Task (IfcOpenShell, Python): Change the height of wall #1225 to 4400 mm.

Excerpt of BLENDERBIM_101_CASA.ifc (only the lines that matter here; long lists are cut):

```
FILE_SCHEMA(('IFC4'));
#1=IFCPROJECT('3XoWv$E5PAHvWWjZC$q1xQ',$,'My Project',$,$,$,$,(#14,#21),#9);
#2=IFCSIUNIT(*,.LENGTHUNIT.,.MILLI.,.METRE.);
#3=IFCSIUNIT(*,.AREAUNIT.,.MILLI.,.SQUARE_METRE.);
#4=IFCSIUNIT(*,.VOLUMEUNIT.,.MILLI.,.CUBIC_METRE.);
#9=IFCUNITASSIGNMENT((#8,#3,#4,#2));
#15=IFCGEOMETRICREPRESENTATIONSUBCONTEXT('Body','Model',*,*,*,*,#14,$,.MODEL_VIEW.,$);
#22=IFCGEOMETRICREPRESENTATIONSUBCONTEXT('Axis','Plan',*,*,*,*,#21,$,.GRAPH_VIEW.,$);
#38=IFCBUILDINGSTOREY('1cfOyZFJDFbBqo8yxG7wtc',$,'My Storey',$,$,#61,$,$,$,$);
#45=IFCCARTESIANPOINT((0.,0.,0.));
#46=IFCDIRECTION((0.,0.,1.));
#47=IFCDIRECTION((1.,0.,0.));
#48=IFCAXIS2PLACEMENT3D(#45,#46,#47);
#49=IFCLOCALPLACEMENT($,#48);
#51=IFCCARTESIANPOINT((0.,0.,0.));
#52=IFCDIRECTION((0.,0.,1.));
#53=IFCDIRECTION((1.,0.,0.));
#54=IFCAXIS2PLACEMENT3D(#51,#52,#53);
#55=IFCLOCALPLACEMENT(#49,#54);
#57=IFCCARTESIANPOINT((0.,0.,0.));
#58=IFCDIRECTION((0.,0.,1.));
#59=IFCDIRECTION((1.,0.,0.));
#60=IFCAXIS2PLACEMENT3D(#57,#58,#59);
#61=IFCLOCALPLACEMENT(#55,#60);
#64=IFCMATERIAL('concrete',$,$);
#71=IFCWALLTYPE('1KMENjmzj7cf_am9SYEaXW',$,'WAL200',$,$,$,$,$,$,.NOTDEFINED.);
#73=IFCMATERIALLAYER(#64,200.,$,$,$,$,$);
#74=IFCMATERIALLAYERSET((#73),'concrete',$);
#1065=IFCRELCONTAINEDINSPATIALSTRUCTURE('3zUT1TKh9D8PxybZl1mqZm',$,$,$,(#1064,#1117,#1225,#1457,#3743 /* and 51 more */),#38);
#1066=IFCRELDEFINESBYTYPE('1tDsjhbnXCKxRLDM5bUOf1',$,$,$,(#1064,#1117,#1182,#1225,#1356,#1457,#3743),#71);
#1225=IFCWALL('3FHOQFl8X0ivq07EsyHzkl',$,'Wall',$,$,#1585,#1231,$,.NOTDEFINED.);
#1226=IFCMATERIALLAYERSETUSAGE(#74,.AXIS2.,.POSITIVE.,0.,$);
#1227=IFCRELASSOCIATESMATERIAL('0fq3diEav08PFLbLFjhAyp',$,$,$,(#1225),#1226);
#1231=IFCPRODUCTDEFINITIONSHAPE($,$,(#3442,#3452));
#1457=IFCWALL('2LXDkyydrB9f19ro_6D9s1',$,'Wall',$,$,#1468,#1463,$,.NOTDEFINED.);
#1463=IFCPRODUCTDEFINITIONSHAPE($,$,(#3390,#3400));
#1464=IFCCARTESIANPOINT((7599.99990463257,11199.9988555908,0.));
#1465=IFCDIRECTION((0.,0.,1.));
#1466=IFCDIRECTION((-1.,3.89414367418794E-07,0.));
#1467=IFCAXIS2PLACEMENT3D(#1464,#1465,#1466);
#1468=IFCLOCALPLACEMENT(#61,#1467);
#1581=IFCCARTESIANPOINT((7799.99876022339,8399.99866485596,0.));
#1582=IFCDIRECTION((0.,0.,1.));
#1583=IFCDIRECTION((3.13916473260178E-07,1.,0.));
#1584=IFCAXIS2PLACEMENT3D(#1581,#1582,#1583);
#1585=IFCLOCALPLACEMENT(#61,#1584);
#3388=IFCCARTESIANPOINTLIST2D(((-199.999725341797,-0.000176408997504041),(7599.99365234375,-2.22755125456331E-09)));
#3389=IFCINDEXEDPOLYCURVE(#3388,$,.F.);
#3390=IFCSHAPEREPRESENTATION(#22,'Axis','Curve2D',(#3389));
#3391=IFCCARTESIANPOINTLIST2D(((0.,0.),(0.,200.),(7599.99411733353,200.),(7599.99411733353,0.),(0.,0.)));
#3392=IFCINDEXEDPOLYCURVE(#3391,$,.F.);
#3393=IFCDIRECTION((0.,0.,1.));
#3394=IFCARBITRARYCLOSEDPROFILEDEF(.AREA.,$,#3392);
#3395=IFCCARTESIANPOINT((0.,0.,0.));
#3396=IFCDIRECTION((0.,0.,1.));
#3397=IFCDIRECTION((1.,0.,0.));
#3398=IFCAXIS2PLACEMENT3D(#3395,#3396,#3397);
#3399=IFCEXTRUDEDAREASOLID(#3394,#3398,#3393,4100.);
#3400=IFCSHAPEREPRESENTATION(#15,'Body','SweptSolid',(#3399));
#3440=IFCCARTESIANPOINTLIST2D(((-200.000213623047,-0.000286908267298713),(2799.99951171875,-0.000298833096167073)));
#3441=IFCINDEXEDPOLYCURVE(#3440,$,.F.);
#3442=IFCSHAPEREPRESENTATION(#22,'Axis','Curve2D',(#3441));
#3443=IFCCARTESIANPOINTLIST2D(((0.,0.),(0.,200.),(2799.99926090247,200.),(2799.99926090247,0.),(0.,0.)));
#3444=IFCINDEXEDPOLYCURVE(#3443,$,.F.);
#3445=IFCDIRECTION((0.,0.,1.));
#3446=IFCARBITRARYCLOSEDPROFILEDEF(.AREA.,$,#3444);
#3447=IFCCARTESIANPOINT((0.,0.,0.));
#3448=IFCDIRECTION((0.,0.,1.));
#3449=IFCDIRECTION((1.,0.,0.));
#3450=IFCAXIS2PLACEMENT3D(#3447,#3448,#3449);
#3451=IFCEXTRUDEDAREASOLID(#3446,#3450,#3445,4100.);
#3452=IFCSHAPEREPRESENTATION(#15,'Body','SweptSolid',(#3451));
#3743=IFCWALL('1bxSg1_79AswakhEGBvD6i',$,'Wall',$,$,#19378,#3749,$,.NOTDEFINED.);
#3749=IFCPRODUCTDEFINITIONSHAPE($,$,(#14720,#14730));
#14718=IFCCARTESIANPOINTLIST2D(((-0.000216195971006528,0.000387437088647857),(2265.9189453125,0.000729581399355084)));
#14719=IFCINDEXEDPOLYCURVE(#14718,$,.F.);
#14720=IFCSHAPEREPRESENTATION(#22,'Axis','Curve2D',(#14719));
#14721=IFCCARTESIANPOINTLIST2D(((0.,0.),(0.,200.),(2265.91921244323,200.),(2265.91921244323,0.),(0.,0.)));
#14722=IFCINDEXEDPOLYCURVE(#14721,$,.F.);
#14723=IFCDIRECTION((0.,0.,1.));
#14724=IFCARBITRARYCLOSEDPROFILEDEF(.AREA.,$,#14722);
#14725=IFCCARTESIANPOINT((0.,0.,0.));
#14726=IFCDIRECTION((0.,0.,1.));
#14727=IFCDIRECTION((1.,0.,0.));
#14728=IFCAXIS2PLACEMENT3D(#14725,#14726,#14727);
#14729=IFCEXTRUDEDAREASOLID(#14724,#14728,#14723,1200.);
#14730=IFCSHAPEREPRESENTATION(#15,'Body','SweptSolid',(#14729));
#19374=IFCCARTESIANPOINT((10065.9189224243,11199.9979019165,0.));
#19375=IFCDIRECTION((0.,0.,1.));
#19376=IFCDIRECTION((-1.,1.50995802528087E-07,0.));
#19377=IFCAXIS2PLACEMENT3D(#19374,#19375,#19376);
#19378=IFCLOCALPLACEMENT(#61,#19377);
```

```python
import ifcopenshell
import ifcopenshell.geom
import ifcopenshell.util.representation
import ifcopenshell.util.shape

model = ifcopenshell.open("BLENDERBIM_101_CASA.ifc")
settings = ifcopenshell.geom.settings()


def volume(element):
    """Net volume in cubic metres, openings subtracted."""
    shape = ifcopenshell.geom.create_shape(settings, element)
    return ifcopenshell.util.shape.get_volume(shape.geometry)


wall = model.by_guid("3FHOQFl8X0ivq07EsyHzkl")
before = volume(wall)

body = ifcopenshell.util.representation.get_representation(wall, "Model", "Body")
solid = body.Items[0]
old_height = solid.Depth
solid.Depth = 4400.0
after = volume(wall)

print(f"height {old_height:g} -> {solid.Depth:g}, volume {before:.3f} -> {after:.3f} m3")

model.write("BLENDERBIM_101_CASA_edited.ifc")
```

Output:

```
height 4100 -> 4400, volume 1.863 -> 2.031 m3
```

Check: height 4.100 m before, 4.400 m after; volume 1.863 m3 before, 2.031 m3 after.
